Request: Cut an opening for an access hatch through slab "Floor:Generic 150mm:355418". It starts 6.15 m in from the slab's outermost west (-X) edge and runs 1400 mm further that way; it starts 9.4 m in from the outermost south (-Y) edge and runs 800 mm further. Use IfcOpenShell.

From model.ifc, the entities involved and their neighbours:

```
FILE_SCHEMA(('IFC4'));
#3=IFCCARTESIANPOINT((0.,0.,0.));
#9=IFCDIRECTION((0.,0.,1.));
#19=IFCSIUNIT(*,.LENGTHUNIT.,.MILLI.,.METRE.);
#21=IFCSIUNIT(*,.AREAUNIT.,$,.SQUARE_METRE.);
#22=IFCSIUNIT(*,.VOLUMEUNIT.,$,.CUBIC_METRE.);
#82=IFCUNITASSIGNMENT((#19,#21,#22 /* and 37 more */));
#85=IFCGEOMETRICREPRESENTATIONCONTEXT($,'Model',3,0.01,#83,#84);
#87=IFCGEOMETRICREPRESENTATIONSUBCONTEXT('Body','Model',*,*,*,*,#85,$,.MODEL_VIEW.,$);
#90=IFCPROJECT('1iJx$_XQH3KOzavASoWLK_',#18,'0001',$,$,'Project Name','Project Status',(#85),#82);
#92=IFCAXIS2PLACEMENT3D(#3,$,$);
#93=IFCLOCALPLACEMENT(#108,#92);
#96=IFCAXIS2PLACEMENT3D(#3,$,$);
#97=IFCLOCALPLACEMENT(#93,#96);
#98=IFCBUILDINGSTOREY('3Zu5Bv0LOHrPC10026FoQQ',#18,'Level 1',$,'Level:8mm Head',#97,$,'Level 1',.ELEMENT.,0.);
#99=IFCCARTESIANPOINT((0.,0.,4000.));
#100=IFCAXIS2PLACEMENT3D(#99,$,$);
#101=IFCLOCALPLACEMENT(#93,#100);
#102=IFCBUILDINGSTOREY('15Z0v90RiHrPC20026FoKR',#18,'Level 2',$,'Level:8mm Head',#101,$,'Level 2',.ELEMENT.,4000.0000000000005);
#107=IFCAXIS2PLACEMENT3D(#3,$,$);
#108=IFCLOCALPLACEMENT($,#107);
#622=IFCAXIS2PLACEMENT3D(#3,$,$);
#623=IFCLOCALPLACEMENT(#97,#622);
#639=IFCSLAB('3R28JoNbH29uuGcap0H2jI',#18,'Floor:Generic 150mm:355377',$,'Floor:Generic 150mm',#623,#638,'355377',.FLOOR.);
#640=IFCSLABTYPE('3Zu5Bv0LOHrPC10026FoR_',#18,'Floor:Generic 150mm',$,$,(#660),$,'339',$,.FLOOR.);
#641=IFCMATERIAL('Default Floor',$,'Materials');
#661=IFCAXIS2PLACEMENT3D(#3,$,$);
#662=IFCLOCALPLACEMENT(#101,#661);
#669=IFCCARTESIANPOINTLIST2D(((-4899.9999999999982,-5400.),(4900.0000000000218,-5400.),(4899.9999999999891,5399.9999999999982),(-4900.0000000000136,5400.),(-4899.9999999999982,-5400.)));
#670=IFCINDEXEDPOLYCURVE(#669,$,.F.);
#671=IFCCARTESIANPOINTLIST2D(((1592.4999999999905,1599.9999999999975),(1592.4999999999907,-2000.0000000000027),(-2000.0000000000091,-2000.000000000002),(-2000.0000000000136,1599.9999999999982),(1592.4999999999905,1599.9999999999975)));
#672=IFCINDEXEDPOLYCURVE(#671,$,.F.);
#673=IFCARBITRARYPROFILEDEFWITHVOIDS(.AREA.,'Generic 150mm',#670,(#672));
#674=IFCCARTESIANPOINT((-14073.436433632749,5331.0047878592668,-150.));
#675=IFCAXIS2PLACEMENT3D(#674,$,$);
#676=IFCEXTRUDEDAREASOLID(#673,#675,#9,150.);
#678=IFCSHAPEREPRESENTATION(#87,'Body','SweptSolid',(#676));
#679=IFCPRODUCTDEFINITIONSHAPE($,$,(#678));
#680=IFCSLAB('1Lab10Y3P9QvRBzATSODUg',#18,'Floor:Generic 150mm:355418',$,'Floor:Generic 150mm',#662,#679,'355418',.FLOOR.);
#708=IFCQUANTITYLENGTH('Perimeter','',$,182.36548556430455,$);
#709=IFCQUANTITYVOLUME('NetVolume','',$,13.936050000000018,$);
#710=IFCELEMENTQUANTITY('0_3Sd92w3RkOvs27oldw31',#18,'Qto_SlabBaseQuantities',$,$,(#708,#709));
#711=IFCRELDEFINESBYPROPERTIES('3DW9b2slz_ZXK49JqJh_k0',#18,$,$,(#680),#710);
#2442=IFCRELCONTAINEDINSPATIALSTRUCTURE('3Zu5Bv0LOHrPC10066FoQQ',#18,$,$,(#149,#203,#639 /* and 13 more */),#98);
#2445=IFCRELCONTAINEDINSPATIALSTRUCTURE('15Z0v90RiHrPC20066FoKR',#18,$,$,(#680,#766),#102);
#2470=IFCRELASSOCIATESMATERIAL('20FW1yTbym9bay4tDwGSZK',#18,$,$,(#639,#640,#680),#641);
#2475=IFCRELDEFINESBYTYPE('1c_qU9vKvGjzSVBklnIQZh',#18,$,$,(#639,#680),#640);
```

```python
import numpy as np
import ifcopenshell
import ifcopenshell.api.feature
import ifcopenshell.api.geometry
import ifcopenshell.api.pset
import ifcopenshell.api.root
import ifcopenshell.geom
import ifcopenshell.util.element
import ifcopenshell.util.placement
import ifcopenshell.util.representation
import ifcopenshell.util.shape
import ifcopenshell.util.unit

model = ifcopenshell.open("model.ifc")
unit_scale = ifcopenshell.util.unit.calculate_unit_scale(model)
volume_scale = ifcopenshell.util.unit.calculate_unit_scale(model, "VOLUMEUNIT")
settings = ifcopenshell.geom.settings()


def volume(element):
    """Net volume in cubic metres, openings subtracted."""
    shape = ifcopenshell.geom.create_shape(settings, element)
    return ifcopenshell.util.shape.get_volume(shape.geometry)


slab = model.by_id(680)
before = volume(slab)

# Extent in the slab's own axes, in metres. The edges named are its -X and -Y sides.
slab_shape = ifcopenshell.geom.create_shape(settings, slab)
vertices = ifcopenshell.util.shape.get_vertices(slab_shape.geometry)
x_min, y_min, bottom = vertices.min(axis=0)
top = vertices[:, 2].max()

opening = ifcopenshell.api.root.create_entity(model, ifc_class="IfcOpeningElement", name="Access hatch opening", predefined_type="OPENING")
context = ifcopenshell.util.representation.get_context(model, "Model", "Body", "MODEL_VIEW")
width, depth = 1.4, 0.8
outline = [(0.0, 0.0), (width, 0.0), (width, depth), (0.0, depth), (0.0, 0.0)]
# Overshoot both faces by 50 mm so the cut is clean.
shape = ifcopenshell.api.geometry.add_slab_representation(
    model, context=context, depth=top - bottom + 0.1, polyline=outline
)
ifcopenshell.api.geometry.assign_representation(model, product=opening, representation=shape)

matrix = ifcopenshell.util.placement.get_local_placement(slab.ObjectPlacement)
matrix[:, 3] = matrix @ np.append(np.array([x_min + 6.15, y_min + 9.4, bottom - 0.05]) / unit_scale, 1.0)
ifcopenshell.api.geometry.edit_object_placement(model, product=opening, matrix=matrix, is_si=False)
ifcopenshell.api.feature.add_feature(model, feature=opening, element=slab)

after = volume(slab)

# Update the slab's stored quantities.
qto = model.by_id(ifcopenshell.util.element.get_pset(slab, "Qto_SlabBaseQuantities", should_inherit=False)["id"])
ifcopenshell.api.pset.edit_qto(model, qto=qto, properties={"NetVolume": after / volume_scale})

print(f"slab volume {before:.3f} -> {after:.3f} m3")

model.write("model_rev.ifc")
```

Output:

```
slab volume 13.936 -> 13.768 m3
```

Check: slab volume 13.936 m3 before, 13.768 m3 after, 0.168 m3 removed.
